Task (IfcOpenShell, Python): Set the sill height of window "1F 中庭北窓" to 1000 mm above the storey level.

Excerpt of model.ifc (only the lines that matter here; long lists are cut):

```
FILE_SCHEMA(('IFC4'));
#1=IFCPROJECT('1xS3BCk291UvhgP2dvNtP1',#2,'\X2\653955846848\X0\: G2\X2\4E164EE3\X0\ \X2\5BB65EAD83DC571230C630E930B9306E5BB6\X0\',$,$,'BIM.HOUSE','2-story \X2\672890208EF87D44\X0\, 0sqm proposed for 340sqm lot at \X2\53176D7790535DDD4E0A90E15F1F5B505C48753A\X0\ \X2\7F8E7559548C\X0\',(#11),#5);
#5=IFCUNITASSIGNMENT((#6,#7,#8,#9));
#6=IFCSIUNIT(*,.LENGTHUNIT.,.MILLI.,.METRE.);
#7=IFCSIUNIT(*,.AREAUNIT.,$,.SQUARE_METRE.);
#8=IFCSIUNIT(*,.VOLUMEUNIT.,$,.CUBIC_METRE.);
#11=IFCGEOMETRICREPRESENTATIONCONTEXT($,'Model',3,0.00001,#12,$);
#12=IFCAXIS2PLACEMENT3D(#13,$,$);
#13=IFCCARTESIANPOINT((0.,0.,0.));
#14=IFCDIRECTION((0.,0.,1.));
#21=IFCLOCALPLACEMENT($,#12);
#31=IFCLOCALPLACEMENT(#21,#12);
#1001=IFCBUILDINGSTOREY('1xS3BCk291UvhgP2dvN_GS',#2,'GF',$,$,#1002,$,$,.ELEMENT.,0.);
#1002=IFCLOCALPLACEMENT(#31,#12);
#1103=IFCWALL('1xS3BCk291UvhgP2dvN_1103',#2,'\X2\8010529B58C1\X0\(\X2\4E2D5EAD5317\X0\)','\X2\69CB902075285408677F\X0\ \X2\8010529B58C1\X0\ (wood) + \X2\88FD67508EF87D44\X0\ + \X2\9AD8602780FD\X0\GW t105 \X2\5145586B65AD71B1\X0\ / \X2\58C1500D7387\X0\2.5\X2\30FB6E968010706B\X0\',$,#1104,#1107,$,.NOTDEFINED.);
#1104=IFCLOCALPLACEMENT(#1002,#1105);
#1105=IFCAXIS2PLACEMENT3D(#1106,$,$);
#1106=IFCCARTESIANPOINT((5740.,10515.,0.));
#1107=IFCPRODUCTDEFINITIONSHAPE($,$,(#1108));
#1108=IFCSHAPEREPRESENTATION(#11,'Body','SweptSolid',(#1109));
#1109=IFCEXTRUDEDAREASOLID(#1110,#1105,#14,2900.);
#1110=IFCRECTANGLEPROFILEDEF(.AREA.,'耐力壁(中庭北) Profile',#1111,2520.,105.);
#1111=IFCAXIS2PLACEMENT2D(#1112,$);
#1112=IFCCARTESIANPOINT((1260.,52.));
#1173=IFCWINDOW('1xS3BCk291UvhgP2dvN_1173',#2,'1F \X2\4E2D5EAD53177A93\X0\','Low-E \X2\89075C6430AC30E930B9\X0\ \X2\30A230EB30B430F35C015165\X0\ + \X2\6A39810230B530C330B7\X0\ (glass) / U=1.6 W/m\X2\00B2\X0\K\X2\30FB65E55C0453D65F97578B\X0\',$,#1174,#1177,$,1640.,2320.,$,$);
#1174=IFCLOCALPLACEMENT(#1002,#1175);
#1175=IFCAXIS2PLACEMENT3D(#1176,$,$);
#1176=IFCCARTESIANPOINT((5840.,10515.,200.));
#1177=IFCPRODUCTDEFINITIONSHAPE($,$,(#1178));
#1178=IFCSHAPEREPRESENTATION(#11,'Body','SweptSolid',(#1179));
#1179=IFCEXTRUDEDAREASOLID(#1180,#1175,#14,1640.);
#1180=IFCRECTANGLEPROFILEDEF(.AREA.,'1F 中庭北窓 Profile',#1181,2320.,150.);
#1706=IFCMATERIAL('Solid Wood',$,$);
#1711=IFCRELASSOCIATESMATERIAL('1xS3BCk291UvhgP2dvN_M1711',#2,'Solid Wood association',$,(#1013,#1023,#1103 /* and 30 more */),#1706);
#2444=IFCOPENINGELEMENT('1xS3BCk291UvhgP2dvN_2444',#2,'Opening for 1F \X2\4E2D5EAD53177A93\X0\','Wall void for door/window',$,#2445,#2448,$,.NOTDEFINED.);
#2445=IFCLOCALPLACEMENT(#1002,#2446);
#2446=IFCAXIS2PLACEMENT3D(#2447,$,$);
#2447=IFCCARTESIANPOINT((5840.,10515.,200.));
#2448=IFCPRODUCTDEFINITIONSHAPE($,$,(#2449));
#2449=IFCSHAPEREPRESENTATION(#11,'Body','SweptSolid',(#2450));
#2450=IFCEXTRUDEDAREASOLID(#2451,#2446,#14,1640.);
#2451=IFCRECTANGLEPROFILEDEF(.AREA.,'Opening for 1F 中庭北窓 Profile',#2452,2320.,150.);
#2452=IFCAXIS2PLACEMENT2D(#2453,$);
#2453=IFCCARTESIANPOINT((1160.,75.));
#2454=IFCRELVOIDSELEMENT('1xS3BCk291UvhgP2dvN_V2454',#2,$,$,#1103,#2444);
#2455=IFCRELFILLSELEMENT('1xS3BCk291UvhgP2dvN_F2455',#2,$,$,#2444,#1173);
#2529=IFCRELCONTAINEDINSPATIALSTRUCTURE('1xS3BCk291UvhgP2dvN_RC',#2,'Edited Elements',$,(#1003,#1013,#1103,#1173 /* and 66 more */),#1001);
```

```python
import numpy as np
import ifcopenshell
import ifcopenshell.api.geometry
import ifcopenshell.geom
import ifcopenshell.util.element
import ifcopenshell.util.placement
import ifcopenshell.util.shape
import ifcopenshell.util.unit

model = ifcopenshell.open("model.ifc")
unit_scale = ifcopenshell.util.unit.calculate_unit_scale(model)

window = model.by_guid("1xS3BCk291UvhgP2dvN_1173")
opening = window.FillsVoids[0].RelatingOpeningElement
storey = ifcopenshell.util.element.get_container(window, ifc_class="IfcBuildingStorey")
level = ifcopenshell.util.placement.get_local_placement(storey.ObjectPlacement)[2, 3]

# The opening's origin need not be at the sill, so measure its lowest point.
shape = ifcopenshell.geom.create_shape(ifcopenshell.geom.settings(), opening)
bottom = ifcopenshell.util.shape.get_shape_bottom_elevation(shape, shape.geometry) / unit_scale
dz = level + 1 / unit_scale - bottom

shift = np.array([0.0, 0.0, dz])
# The window is not placed relative to its opening, so move both.
for product in (opening, window):
    matrix = ifcopenshell.util.placement.get_local_placement(product.ObjectPlacement)
    matrix[:3, 3] += shift
    ifcopenshell.api.geometry.edit_object_placement(model, product=product, matrix=matrix, is_si=False)

print(f"moved by {dz * unit_scale:+.3f} m")

model.write("model_v2.ifc")
```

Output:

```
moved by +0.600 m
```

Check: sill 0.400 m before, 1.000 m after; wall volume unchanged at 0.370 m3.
